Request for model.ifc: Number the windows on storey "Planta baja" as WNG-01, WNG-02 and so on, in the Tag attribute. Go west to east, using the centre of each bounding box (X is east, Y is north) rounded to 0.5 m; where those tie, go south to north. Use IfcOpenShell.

First a look at what the model holds.

```python
import ifcopenshell
import ifcopenshell.util.element
import ifcopenshell.util.placement

model = ifcopenshell.open("model.ifc")
print(model.schema)
storey = next(s for s in model.by_type("IfcBuildingStorey") if s.Name == "Planta baja")
windows = [e for e in ifcopenshell.util.element.get_decomposition(storey) if e.is_a("IfcWindow")]
for e in sorted(windows, key=lambda e: e.id()):
    origin = ifcopenshell.util.placement.get_local_placement(e.ObjectPlacement)[:3, 3]
    print(e.id(), e.Tag, e.Name, origin.round(2) + 0.0, sep=" | ")
```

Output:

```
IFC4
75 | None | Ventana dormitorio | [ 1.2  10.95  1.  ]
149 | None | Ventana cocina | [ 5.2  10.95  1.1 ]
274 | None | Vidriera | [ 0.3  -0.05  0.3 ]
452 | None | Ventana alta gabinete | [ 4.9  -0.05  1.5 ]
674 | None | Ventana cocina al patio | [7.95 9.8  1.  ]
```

```python
import ifcopenshell
import ifcopenshell.geom
import ifcopenshell.util.element
import ifcopenshell.util.shape

model = ifcopenshell.open("model.ifc")
settings = ifcopenshell.geom.settings()
settings.set("use-world-coords", True)


def centre(element):
    shape = ifcopenshell.geom.create_shape(settings, element)
    return ifcopenshell.util.shape.get_bbox_centroid(shape.geometry)


storey = next(s for s in model.by_type("IfcBuildingStorey") if s.Name == "Planta baja")
windows = [e for e in ifcopenshell.util.element.get_decomposition(storey) if e.is_a("IfcWindow")]

# Insertion points can sit at a corner or the storey origin, so sort by the geometry (in metres).
centres = {e: centre(e) for e in windows}
windows.sort(key=lambda e: (round(centres[e][0] / 0.5), centres[e][1]))

for i, e in enumerate(windows, start=1):
    number = f"WNG-{i:02d}"
    e.Tag = number
    print(e.id(), number)

model.write("model_v2.ifc")
```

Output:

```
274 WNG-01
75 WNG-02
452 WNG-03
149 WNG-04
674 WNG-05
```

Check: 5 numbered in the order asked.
